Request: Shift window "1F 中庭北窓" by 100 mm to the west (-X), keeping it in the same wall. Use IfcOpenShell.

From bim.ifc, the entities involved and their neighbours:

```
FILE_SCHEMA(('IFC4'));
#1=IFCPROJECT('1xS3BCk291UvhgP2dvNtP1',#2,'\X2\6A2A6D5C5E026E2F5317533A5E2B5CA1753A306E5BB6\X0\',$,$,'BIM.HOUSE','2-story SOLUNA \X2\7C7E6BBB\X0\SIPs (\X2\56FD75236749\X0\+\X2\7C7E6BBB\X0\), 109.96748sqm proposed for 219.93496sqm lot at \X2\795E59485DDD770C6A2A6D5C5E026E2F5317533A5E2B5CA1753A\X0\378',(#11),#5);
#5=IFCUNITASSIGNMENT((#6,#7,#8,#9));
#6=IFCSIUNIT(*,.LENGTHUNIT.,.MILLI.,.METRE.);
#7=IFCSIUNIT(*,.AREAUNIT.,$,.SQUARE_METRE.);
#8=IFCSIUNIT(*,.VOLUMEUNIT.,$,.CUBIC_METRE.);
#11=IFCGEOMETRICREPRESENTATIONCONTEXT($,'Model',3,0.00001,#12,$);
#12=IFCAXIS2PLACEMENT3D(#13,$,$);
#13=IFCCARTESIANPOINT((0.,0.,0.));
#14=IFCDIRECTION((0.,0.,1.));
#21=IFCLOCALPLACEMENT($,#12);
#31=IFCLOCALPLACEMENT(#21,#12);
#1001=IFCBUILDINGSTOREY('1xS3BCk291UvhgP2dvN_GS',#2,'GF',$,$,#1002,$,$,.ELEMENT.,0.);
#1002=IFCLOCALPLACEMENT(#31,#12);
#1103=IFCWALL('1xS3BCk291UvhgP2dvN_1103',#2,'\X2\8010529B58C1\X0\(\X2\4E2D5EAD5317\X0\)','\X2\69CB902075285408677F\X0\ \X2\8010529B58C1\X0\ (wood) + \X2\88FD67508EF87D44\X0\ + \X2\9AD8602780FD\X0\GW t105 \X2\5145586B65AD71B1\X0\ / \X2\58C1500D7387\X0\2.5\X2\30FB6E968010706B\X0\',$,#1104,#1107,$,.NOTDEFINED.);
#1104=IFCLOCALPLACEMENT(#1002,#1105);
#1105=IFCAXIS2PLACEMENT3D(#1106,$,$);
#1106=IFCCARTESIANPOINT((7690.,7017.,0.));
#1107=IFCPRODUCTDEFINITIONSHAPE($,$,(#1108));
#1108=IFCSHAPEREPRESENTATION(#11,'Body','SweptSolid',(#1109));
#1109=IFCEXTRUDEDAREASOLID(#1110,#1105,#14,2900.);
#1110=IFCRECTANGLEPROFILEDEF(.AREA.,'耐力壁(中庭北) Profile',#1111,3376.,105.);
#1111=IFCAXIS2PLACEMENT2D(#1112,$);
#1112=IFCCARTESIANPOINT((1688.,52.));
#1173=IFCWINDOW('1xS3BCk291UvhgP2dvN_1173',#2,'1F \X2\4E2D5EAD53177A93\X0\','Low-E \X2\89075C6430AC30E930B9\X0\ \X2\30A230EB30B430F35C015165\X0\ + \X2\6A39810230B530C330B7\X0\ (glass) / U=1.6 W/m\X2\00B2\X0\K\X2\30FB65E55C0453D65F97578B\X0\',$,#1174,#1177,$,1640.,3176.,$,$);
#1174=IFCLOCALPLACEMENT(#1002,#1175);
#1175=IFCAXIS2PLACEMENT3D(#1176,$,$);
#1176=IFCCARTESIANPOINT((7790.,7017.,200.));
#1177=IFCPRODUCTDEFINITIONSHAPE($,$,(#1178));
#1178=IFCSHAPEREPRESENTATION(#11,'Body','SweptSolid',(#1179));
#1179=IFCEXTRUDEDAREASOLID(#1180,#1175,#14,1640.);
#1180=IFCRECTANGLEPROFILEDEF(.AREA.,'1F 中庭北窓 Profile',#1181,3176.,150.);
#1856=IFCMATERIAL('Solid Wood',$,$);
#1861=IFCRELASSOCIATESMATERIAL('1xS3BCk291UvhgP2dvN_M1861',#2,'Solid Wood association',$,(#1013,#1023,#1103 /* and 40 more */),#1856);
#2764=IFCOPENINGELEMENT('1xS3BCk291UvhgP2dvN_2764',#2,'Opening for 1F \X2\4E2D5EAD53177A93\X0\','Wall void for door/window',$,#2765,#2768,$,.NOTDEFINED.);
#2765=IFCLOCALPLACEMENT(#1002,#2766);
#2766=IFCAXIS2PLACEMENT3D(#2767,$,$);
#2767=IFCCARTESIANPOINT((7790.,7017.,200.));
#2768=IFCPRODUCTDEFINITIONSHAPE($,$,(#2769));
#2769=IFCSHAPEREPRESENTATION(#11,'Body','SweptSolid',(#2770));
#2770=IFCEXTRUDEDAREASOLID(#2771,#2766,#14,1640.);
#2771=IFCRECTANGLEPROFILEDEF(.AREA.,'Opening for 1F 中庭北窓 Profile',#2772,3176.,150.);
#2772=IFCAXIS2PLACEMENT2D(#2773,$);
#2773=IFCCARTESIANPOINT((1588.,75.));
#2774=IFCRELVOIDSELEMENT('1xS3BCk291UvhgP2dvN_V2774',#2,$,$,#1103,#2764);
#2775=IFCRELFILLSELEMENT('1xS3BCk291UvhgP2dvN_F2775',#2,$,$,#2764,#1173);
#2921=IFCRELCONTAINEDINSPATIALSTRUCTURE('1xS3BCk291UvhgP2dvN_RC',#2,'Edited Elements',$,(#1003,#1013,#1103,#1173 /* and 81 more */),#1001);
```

```python
import ifcopenshell
import ifcopenshell.api.geometry
import ifcopenshell.util.placement

model = ifcopenshell.open("bim.ifc")

window = model.by_guid("1xS3BCk291UvhgP2dvN_1173")
opening = window.FillsVoids[0].RelatingOpeningElement
wall = opening.VoidsElements[0].RelatingBuildingElement

wall_matrix = ifcopenshell.util.placement.get_local_placement(wall.ObjectPlacement)
shift = wall_matrix[:3, 0] * -100.0
before = ifcopenshell.util.placement.get_local_placement(window.ObjectPlacement)[:3, 3].copy()

# The window is not placed relative to its opening, so move both.
for product in (opening, window):
    matrix = ifcopenshell.util.placement.get_local_placement(product.ObjectPlacement)
    matrix[:3, 3] += shift
    ifcopenshell.api.geometry.edit_object_placement(model, product=product, matrix=matrix, is_si=False)

after = ifcopenshell.util.placement.get_local_placement(window.ObjectPlacement)[:3, 3]
print("window moved by", (after - before).round(3) + 0.0)

model.write("bim-out.ifc")
```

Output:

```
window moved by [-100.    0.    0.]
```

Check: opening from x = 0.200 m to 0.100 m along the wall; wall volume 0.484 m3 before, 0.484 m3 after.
